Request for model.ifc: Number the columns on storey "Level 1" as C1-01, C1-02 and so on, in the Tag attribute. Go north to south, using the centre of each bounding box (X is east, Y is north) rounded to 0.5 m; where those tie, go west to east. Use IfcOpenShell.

First a look at what the model holds.

```python
import ifcopenshell
import ifcopenshell.util.element
import ifcopenshell.util.placement

model = ifcopenshell.open("model.ifc")
print(model.schema)
storey = next(s for s in model.by_type("IfcBuildingStorey") if s.Name == "Level 1")
columns = [e for e in ifcopenshell.util.element.get_decomposition(storey) if e.is_a("IfcColumn")]
for e in sorted(columns, key=lambda e: e.id()):
    origin = ifcopenshell.util.placement.get_local_placement(e.ObjectPlacement)[:3, 3]
    print(e.id(), e.Tag, e.Name, origin.round(2) + 0.0, sep=" | ")
```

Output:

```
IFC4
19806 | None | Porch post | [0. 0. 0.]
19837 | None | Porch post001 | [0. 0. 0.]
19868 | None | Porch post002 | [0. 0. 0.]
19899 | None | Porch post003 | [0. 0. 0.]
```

```python
import ifcopenshell
import ifcopenshell.geom
import ifcopenshell.util.element
import ifcopenshell.util.shape

model = ifcopenshell.open("model.ifc")
settings = ifcopenshell.geom.settings()
settings.set("use-world-coords", True)


def centre(element):
    shape = ifcopenshell.geom.create_shape(settings, element)
    return ifcopenshell.util.shape.get_bbox_centroid(shape.geometry)


storey = next(s for s in model.by_type("IfcBuildingStorey") if s.Name == "Level 1")
columns = [e for e in ifcopenshell.util.element.get_decomposition(storey) if e.is_a("IfcColumn")]

# Insertion points can sit at a corner or the storey origin, so sort by the geometry (in metres).
centres = {e: centre(e) for e in columns}
columns.sort(key=lambda e: (-round(centres[e][1] / 0.5), centres[e][0]))

for i, e in enumerate(columns, start=1):
    number = f"C1-{i:02d}"
    e.Tag = number
    print(e.id(), number)

model.write("model-out.ifc")
```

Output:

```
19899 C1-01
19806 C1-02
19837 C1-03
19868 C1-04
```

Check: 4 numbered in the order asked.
